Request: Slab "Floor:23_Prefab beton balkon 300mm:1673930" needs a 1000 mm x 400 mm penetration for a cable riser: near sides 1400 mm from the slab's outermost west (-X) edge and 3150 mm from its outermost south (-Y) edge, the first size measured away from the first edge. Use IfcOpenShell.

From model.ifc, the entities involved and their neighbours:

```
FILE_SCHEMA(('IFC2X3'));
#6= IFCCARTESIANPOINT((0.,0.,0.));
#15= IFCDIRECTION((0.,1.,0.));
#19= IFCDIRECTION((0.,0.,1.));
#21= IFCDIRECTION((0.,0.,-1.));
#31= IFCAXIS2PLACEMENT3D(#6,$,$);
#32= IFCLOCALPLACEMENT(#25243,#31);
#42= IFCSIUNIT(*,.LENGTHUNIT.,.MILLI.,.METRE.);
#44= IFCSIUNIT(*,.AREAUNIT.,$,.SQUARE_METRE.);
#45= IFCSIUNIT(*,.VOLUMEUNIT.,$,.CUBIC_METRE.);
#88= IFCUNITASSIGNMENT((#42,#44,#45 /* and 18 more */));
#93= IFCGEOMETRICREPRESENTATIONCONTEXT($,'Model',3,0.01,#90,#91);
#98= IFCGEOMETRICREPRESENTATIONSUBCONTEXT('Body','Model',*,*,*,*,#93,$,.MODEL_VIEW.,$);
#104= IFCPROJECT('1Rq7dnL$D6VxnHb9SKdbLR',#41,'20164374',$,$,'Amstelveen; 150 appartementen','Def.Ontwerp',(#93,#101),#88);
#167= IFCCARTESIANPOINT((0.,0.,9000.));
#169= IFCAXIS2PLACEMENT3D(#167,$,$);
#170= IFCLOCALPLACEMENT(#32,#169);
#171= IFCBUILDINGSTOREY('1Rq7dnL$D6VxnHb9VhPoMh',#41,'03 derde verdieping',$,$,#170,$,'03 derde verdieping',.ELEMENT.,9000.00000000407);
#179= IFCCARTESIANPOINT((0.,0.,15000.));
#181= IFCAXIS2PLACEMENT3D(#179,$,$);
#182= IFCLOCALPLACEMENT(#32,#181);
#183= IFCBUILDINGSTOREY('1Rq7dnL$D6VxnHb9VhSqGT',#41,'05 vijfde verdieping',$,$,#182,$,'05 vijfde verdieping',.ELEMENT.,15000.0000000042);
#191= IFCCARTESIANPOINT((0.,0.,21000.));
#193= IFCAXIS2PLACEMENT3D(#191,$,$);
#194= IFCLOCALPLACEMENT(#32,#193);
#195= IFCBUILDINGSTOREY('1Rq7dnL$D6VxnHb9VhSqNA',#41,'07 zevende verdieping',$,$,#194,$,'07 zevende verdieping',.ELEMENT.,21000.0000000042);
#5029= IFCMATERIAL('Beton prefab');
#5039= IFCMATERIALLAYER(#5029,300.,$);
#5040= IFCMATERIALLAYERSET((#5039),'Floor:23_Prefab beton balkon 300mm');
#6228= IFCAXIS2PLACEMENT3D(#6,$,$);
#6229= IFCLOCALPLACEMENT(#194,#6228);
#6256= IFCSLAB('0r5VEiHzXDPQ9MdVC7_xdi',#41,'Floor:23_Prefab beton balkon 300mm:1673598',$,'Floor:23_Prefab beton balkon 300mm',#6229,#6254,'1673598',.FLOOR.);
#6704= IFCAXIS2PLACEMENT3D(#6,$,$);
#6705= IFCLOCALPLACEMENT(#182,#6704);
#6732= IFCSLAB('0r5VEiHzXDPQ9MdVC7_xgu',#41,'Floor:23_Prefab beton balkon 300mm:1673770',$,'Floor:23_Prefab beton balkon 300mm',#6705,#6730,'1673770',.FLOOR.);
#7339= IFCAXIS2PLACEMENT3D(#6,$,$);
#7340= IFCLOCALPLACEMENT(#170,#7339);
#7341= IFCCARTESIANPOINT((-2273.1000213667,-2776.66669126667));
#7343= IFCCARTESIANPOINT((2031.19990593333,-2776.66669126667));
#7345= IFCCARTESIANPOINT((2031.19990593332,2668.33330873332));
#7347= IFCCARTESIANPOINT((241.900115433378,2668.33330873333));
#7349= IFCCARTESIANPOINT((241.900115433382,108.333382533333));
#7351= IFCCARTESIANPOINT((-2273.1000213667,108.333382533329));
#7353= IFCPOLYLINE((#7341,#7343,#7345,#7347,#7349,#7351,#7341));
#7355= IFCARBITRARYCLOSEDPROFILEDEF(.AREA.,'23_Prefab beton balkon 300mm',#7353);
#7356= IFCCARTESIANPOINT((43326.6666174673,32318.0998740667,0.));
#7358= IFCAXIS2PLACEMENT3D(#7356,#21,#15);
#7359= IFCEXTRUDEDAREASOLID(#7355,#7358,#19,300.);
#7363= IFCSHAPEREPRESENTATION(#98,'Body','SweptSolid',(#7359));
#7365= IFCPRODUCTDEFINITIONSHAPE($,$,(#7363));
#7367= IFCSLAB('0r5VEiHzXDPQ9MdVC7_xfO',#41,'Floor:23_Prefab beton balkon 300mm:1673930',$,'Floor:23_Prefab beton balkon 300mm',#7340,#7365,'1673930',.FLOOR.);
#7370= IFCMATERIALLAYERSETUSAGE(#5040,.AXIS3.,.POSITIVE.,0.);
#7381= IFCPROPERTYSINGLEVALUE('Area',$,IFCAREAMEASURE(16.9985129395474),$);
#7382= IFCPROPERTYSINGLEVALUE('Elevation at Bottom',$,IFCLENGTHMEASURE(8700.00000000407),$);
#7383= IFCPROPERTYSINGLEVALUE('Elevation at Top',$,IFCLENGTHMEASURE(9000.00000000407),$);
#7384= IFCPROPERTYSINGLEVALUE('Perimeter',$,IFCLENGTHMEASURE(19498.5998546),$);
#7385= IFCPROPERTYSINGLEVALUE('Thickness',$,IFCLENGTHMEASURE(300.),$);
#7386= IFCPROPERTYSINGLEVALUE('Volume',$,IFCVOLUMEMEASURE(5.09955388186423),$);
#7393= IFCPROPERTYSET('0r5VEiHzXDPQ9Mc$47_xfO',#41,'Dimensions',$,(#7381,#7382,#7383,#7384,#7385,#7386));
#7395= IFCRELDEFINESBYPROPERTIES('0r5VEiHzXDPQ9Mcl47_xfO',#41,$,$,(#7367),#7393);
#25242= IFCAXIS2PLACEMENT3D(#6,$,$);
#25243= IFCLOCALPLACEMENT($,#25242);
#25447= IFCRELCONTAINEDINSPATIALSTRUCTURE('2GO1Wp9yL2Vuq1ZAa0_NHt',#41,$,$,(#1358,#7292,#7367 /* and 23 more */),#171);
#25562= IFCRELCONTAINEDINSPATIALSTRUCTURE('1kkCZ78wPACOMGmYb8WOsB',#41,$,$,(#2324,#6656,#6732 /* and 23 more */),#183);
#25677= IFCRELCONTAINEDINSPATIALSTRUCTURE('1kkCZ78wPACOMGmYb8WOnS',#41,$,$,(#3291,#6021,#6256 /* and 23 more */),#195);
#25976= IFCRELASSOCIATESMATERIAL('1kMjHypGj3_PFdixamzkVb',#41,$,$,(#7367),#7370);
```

```python
import numpy as np
import ifcopenshell
import ifcopenshell.api.feature
import ifcopenshell.api.geometry
import ifcopenshell.api.pset
import ifcopenshell.api.root
import ifcopenshell.geom
import ifcopenshell.util.element
import ifcopenshell.util.placement
import ifcopenshell.util.representation
import ifcopenshell.util.shape
import ifcopenshell.util.unit

model = ifcopenshell.open("model.ifc")
unit_scale = ifcopenshell.util.unit.calculate_unit_scale(model)
area_scale = ifcopenshell.util.unit.calculate_unit_scale(model, "AREAUNIT")
volume_scale = ifcopenshell.util.unit.calculate_unit_scale(model, "VOLUMEUNIT")
settings = ifcopenshell.geom.settings()


def volume(element):
    """Net volume in cubic metres, openings subtracted."""
    shape = ifcopenshell.geom.create_shape(settings, element)
    return ifcopenshell.util.shape.get_volume(shape.geometry)


slab = model.by_id(7367)
before = volume(slab)

# Extent in the slab's own axes, in metres. The edges named are its -X and -Y sides.
slab_shape = ifcopenshell.geom.create_shape(settings, slab)
vertices = ifcopenshell.util.shape.get_vertices(slab_shape.geometry)
x_min, y_min, bottom = vertices.min(axis=0)
top = vertices[:, 2].max()

opening = ifcopenshell.api.root.create_entity(model, ifc_class="IfcOpeningElement", name="Cable riser opening")
context = ifcopenshell.util.representation.get_context(model, "Model", "Body", "MODEL_VIEW")
width, depth = 1, 0.4
outline = [(0.0, 0.0), (width, 0.0), (width, depth), (0.0, depth), (0.0, 0.0)]
# Overshoot both faces by 50 mm so the cut is clean.
shape = ifcopenshell.api.geometry.add_slab_representation(
    model, context=context, depth=top - bottom + 0.1, polyline=outline
)
ifcopenshell.api.geometry.assign_representation(model, product=opening, representation=shape)

matrix = ifcopenshell.util.placement.get_local_placement(slab.ObjectPlacement)
matrix[:, 3] = matrix @ np.append(np.array([x_min + 1.4, y_min + 3.15, bottom - 0.05]) / unit_scale, 1.0)
ifcopenshell.api.geometry.edit_object_placement(model, product=opening, matrix=matrix, is_si=False)
ifcopenshell.api.feature.add_feature(model, feature=opening, element=slab)

after = volume(slab)

# Update the slab's stored quantities.
pset = model.by_id(ifcopenshell.util.element.get_pset(slab, "Dimensions", should_inherit=False)["id"])
ifcopenshell.api.pset.edit_pset(model, pset=pset, properties={
    "Area": model.create_entity("IfcAreaMeasure", after / (top - bottom) / area_scale),
    "Volume": model.create_entity("IfcVolumeMeasure", after / volume_scale),
})

print(f"slab volume {before:.3f} -> {after:.3f} m3")

model.write("model_updated.ifc")
```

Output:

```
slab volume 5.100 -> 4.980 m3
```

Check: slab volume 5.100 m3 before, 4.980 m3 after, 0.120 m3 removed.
